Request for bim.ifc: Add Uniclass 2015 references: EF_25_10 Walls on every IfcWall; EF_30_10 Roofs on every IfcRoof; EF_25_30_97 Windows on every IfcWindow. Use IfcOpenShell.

First a look at what the model holds.

```python
import ifcopenshell

model = ifcopenshell.open("bim.ifc")
print(model.schema)
print("classifications:", [c.Name for c in model.by_type("IfcClassification")])
for ifc_class in ("IfcDoor", "IfcRoof", "IfcStair", "IfcWall", "IfcWindow"):
    print(ifc_class, len(model.by_type(ifc_class)))
```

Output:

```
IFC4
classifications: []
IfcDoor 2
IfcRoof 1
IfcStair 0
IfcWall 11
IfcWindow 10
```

```python
import ifcopenshell
import ifcopenshell.api.classification

model = ifcopenshell.open("bim.ifc")

system = ifcopenshell.api.classification.add_classification(model, classification="Uniclass 2015")

codes = {
    "IfcWall": ("EF_25_10", "Walls"),
    "IfcRoof": ("EF_30_10", "Roofs"),
    "IfcWindow": ("EF_25_30_97", "Windows"),
}
for ifc_class, (code, name) in codes.items():
    products = model.by_type(ifc_class)
    ifcopenshell.api.classification.add_reference(
        model, products=products, classification=system, identification=code, name=name
    )
    print(code, len(products))

model.write("bim_rev.ifc")
```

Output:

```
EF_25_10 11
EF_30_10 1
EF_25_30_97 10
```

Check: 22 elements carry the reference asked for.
